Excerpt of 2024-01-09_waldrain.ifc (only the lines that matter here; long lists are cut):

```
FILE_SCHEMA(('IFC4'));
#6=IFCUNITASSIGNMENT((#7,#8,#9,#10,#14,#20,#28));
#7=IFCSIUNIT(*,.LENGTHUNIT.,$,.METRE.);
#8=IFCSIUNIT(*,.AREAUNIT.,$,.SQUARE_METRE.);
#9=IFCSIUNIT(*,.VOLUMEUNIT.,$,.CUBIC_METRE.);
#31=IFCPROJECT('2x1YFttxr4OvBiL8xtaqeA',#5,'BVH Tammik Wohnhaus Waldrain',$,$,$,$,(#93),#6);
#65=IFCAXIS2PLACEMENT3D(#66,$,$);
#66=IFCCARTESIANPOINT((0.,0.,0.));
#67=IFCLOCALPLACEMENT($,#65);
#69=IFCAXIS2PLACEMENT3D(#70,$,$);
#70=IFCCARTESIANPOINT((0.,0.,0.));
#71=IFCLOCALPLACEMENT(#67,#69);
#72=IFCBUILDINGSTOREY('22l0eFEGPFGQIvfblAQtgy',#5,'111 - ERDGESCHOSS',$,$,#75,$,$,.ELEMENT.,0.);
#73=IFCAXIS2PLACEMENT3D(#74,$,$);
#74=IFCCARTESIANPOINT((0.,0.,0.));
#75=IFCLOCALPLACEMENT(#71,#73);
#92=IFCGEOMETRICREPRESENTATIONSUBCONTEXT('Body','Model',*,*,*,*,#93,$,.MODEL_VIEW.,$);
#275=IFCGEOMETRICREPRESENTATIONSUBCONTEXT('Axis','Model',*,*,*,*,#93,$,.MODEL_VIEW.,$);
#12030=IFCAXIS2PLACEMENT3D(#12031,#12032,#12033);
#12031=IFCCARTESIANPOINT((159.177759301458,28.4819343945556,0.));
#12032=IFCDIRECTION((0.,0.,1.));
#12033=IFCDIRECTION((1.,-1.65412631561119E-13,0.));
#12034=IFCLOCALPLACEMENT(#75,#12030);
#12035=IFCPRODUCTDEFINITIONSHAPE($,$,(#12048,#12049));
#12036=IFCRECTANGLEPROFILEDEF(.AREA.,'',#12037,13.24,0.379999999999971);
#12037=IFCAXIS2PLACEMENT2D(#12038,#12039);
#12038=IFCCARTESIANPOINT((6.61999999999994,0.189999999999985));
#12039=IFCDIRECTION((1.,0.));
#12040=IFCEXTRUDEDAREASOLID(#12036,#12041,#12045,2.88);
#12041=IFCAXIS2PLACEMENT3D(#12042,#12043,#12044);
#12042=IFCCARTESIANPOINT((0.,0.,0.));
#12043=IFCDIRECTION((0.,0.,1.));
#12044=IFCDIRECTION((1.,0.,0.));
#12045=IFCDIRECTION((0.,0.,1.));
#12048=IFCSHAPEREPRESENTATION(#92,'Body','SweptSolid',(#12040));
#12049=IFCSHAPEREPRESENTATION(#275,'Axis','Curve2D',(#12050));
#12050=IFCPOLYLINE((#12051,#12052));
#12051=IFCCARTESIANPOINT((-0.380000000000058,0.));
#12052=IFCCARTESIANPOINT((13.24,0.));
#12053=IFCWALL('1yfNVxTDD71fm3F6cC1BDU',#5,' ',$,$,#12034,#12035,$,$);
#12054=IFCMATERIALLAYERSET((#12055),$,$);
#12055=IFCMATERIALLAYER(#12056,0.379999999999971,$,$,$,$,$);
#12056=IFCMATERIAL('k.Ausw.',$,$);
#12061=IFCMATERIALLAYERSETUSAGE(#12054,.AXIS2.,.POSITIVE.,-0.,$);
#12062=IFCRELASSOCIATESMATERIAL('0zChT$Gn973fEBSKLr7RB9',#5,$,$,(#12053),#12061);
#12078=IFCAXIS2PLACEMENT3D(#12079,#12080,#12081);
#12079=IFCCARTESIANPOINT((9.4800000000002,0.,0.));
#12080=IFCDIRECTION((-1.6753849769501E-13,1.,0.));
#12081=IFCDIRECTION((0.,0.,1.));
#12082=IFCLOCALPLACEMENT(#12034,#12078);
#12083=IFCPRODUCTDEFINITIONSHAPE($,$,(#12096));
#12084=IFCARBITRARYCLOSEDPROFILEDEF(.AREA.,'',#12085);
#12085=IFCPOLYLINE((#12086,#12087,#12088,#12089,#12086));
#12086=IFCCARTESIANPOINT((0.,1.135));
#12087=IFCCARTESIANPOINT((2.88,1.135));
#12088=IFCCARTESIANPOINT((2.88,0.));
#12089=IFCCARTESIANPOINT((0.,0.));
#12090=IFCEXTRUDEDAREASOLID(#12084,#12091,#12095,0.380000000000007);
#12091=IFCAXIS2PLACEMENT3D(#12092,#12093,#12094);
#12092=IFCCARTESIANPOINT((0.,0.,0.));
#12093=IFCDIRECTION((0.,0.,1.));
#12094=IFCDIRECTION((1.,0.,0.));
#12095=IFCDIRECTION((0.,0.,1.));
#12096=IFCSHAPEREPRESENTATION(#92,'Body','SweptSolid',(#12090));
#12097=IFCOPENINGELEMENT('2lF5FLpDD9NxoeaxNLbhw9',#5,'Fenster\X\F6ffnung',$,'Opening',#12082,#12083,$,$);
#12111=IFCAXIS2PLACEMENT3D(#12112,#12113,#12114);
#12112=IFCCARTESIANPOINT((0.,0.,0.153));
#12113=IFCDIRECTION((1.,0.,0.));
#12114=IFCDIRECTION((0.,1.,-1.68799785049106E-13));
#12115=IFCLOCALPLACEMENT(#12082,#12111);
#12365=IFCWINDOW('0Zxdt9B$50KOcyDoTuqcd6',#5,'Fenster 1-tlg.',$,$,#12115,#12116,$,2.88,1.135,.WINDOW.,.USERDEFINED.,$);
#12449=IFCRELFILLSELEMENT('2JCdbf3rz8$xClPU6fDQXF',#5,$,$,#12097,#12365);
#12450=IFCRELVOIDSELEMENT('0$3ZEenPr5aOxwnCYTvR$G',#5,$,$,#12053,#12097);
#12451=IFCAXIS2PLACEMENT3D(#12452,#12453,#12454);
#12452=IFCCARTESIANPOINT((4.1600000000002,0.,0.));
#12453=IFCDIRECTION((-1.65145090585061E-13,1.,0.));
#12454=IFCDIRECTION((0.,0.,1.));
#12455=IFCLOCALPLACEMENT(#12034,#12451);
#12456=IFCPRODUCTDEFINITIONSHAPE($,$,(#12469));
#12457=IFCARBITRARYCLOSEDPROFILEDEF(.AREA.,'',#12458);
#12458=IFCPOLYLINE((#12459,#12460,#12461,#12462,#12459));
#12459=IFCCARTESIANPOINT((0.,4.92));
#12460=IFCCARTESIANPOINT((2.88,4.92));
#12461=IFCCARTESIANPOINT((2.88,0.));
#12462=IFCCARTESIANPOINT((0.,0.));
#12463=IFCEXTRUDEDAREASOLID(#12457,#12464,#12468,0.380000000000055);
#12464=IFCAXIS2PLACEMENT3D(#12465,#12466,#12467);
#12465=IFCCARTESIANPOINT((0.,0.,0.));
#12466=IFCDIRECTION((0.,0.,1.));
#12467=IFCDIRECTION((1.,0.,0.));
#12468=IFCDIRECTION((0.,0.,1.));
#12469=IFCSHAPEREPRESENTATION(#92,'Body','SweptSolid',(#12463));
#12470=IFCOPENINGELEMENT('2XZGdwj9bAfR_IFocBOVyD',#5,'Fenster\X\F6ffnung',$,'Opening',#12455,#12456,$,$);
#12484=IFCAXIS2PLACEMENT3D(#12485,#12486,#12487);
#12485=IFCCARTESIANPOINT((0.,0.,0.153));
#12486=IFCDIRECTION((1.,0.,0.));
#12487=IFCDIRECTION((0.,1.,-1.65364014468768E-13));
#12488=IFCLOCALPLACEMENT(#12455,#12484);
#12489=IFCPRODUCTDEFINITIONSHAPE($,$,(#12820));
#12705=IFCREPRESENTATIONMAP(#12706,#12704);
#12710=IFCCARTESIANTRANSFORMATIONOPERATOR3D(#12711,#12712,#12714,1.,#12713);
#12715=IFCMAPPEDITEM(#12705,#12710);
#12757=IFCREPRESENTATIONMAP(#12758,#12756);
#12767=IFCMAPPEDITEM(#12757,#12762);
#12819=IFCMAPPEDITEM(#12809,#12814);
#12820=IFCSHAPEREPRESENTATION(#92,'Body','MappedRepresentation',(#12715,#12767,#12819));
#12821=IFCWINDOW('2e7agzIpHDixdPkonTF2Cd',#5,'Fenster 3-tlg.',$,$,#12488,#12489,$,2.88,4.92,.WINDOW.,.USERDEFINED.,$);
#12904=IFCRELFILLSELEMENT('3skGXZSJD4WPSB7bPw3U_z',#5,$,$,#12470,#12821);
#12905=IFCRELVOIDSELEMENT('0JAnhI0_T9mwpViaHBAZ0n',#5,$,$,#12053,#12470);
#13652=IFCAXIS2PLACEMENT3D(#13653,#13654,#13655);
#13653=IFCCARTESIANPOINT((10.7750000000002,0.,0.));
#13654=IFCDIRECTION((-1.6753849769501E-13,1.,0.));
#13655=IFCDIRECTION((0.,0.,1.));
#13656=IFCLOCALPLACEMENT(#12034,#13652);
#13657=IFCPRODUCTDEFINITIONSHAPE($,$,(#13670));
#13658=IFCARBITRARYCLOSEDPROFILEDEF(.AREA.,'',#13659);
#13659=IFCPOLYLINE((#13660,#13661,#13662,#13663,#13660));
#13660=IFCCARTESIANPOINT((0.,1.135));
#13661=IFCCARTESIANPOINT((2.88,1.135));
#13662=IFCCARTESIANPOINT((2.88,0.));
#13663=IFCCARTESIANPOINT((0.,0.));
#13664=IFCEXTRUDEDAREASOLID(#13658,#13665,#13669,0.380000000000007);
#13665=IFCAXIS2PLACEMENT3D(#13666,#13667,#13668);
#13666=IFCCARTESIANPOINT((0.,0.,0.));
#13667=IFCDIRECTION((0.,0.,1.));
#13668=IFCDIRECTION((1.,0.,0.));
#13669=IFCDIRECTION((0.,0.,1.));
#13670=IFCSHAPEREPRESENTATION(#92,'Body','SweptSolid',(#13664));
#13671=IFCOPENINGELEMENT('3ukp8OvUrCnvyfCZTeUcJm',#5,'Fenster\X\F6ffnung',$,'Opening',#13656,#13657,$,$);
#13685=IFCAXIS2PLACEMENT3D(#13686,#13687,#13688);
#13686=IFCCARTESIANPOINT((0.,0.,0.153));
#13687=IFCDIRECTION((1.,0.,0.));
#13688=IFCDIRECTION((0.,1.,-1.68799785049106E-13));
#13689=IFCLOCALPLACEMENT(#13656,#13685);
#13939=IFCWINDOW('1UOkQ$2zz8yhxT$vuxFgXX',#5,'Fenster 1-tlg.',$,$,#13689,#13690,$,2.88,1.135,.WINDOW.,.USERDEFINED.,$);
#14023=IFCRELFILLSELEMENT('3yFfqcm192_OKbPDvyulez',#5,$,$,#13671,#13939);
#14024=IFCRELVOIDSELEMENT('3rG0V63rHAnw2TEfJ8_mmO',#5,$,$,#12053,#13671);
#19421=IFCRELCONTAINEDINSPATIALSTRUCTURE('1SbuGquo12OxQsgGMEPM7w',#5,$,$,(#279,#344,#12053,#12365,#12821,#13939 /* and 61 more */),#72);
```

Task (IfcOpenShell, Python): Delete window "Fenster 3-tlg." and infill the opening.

```python
import ifcopenshell
import ifcopenshell.api.feature
import ifcopenshell.api.root
import ifcopenshell.geom
import ifcopenshell.util.shape

model = ifcopenshell.open("2024-01-09_waldrain.ifc")
settings = ifcopenshell.geom.settings()


def volume(element):
    """Net volume in cubic metres, openings subtracted."""
    shape = ifcopenshell.geom.create_shape(settings, element)
    return ifcopenshell.util.shape.get_volume(shape.geometry)


window = model.by_guid("2e7agzIpHDixdPkonTF2Cd")
opening = window.FillsVoids[0].RelatingOpeningElement
wall = opening.VoidsElements[0].RelatingBuildingElement
before = volume(wall)

ifcopenshell.api.root.remove_product(model, product=window)
ifcopenshell.api.feature.remove_feature(model, feature=opening)

after = volume(wall)

print(f"wall volume {before:.3f} -> {after:.3f} m3")

model.write("2024-01-09_waldrain_updated.ifc")
```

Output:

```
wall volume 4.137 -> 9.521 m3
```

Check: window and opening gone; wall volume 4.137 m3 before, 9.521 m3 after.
